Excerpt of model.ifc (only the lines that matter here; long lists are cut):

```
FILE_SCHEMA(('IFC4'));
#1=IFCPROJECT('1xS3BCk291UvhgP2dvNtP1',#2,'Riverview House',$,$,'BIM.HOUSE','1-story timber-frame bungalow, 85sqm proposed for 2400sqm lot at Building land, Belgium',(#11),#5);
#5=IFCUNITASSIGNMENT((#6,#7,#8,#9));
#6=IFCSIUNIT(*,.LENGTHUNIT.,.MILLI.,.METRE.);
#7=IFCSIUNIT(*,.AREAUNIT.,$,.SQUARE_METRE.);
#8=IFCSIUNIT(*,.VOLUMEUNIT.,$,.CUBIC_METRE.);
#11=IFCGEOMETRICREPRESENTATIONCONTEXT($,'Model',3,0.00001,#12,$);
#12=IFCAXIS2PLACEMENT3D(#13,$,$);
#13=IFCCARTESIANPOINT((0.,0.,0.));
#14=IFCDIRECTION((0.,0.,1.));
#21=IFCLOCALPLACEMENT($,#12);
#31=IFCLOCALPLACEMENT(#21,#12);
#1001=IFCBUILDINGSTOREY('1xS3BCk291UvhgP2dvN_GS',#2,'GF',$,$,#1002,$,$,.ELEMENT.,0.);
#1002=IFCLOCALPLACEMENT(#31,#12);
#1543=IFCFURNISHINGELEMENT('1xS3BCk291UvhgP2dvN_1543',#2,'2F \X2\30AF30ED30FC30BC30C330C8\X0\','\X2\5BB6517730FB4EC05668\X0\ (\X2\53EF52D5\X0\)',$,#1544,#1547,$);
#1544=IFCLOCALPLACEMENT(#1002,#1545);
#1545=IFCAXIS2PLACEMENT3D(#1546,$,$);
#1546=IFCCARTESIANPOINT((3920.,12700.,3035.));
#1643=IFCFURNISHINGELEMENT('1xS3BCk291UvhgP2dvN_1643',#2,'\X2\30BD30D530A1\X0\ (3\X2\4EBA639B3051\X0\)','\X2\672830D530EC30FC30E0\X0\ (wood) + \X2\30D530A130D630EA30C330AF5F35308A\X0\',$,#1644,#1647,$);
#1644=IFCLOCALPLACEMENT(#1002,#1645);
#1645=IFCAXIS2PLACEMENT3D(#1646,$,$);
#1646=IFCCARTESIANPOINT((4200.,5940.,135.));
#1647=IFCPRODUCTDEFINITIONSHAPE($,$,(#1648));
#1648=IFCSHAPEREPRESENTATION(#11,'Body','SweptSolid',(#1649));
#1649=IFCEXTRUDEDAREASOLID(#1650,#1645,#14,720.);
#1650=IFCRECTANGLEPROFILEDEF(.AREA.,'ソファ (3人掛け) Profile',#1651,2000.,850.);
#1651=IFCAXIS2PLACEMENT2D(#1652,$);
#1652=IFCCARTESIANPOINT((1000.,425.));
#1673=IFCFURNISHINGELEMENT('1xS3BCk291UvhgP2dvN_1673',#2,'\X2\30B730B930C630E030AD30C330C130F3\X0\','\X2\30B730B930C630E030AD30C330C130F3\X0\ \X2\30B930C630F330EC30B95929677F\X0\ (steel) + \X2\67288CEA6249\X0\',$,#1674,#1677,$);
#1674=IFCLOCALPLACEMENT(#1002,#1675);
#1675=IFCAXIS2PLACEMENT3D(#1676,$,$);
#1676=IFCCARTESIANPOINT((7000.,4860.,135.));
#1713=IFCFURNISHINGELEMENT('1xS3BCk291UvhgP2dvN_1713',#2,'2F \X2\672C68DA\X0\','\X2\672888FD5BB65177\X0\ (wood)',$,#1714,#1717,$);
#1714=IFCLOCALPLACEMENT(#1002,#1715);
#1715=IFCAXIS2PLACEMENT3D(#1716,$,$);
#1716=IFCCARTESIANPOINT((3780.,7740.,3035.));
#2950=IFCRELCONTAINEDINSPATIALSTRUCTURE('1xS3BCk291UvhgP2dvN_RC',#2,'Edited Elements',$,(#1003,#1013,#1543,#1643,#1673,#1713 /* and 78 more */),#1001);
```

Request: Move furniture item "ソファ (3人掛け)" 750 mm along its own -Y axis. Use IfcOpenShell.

```python
import ifcopenshell
import ifcopenshell.api.geometry
import ifcopenshell.util.placement
import ifcopenshell.util.unit

model = ifcopenshell.open("model.ifc")
unit_scale = ifcopenshell.util.unit.calculate_unit_scale(model)

item = model.by_guid("1xS3BCk291UvhgP2dvN_1643")
matrix = ifcopenshell.util.placement.get_local_placement(item.ObjectPlacement)
matrix[:3, 3] -= matrix[:3, 1] * 0.75 / unit_scale
ifcopenshell.api.geometry.edit_object_placement(model, product=item, matrix=matrix, is_si=False)

print(ifcopenshell.util.placement.get_local_placement(item.ObjectPlacement).round(3) + 0.0)

model.write("model_v2.ifc")
```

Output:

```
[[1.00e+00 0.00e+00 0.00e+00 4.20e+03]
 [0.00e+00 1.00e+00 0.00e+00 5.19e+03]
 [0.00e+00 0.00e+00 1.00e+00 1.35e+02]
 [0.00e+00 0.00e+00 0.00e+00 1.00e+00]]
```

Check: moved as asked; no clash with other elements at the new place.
